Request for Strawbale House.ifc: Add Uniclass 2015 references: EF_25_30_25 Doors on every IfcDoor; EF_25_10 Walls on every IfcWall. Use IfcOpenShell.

First a look at what the model holds.

```python
import ifcopenshell

model = ifcopenshell.open("Strawbale House.ifc")
print(model.schema)
print("classifications:", [c.Name for c in model.by_type("IfcClassification")])
for ifc_class in ("IfcDoor", "IfcRoof", "IfcStair", "IfcWall", "IfcWindow"):
    print(ifc_class, len(model.by_type(ifc_class)))
```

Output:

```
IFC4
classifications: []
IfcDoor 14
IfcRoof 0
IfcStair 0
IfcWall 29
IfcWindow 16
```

```python
import ifcopenshell
import ifcopenshell.api.classification

model = ifcopenshell.open("Strawbale House.ifc")

system = ifcopenshell.api.classification.add_classification(model, classification="Uniclass 2015")

codes = {
    "IfcDoor": ("EF_25_30_25", "Doors"),
    "IfcWall": ("EF_25_10", "Walls"),
}
for ifc_class, (code, name) in codes.items():
    products = model.by_type(ifc_class)
    ifcopenshell.api.classification.add_reference(
        model, products=products, classification=system, identification=code, name=name
    )
    print(code, len(products))

model.write("Strawbale House_rev.ifc")
```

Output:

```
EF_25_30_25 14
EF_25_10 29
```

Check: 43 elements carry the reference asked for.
